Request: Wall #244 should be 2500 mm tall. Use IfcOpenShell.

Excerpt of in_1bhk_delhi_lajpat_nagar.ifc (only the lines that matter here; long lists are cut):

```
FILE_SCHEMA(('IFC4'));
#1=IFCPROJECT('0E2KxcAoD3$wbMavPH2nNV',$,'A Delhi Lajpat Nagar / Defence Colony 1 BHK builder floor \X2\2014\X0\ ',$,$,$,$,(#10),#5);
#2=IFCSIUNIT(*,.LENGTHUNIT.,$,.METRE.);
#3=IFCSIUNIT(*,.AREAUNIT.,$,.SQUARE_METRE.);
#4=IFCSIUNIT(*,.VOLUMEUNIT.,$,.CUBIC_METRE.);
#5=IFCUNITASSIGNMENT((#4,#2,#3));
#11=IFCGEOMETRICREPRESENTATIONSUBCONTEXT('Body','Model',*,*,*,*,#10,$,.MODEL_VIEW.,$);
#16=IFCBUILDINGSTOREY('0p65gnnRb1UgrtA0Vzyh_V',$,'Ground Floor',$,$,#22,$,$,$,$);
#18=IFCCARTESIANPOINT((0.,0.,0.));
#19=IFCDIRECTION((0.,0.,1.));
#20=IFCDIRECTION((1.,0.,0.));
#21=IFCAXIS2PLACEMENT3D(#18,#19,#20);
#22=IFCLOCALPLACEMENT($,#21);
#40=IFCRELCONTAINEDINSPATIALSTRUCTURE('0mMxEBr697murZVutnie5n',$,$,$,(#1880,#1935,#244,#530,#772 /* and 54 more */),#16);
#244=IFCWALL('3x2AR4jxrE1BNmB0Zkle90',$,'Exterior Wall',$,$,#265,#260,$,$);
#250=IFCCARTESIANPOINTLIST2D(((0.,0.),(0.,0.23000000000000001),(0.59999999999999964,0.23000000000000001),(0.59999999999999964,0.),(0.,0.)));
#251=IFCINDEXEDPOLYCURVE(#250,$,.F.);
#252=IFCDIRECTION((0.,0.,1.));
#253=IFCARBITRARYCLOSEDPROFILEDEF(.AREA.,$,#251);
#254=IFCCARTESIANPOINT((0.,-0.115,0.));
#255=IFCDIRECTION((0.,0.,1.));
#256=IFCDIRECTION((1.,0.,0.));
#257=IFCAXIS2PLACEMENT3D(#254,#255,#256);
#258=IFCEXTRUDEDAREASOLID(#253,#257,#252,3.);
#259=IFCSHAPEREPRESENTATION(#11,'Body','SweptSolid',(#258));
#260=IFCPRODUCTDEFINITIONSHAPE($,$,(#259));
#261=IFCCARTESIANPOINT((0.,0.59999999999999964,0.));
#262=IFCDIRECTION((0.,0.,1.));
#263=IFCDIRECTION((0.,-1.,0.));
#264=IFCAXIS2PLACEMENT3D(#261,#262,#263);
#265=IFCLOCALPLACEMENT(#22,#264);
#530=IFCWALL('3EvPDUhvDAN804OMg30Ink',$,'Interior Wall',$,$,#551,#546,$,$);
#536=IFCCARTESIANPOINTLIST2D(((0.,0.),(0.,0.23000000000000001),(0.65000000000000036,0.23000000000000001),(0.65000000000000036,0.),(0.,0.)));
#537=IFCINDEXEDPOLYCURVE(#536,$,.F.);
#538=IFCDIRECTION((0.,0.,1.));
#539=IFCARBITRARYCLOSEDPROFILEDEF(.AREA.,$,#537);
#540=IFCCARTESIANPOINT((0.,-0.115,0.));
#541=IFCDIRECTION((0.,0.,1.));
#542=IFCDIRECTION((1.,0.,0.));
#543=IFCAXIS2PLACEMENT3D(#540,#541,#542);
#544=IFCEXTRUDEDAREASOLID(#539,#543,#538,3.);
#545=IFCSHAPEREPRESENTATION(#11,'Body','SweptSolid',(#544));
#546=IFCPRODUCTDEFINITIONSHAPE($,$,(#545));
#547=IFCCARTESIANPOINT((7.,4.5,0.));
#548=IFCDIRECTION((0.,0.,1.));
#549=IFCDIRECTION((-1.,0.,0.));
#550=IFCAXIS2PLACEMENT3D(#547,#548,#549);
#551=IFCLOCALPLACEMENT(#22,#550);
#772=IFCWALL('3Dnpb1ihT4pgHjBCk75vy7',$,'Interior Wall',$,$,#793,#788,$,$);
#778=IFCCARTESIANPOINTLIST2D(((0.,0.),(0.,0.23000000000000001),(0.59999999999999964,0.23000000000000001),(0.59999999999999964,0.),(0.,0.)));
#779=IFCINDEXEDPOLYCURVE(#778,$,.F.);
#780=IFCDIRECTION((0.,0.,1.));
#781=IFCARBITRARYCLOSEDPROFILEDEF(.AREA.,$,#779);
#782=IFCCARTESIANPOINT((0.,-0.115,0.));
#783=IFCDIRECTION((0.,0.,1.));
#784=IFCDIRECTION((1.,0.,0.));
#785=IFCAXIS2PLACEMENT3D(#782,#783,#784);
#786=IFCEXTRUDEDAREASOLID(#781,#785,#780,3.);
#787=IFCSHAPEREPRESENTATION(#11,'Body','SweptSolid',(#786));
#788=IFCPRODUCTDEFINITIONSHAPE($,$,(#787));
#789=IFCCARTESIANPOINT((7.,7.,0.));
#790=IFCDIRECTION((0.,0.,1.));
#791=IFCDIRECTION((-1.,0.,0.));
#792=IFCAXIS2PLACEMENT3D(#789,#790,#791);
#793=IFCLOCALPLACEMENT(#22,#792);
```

```python
import ifcopenshell
import ifcopenshell.geom
import ifcopenshell.util.representation
import ifcopenshell.util.shape
import ifcopenshell.util.unit

model = ifcopenshell.open("in_1bhk_delhi_lajpat_nagar.ifc")
unit_scale = ifcopenshell.util.unit.calculate_unit_scale(model)
settings = ifcopenshell.geom.settings()


def volume(element):
    """Net volume in cubic metres, openings subtracted."""
    shape = ifcopenshell.geom.create_shape(settings, element)
    return ifcopenshell.util.shape.get_volume(shape.geometry)


wall = model.by_guid("3x2AR4jxrE1BNmB0Zkle90")
before = volume(wall)

body = ifcopenshell.util.representation.get_representation(wall, "Model", "Body")
solid = body.Items[0]
old_height = solid.Depth
solid.Depth = 2.5 / unit_scale
after = volume(wall)

print(f"height {old_height:g} -> {solid.Depth:g}, volume {before:.3f} -> {after:.3f} m3")

model.write("in_1bhk_delhi_lajpat_nagar_edited.ifc")
```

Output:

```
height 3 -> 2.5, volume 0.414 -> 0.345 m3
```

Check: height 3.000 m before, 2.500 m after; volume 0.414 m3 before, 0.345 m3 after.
